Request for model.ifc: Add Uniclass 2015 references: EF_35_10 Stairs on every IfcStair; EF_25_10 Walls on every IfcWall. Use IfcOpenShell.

First a look at what the model holds.

```python
import ifcopenshell

model = ifcopenshell.open("model.ifc")
print(model.schema)
print("classifications:", [c.Name for c in model.by_type("IfcClassification")])
for ifc_class in ("IfcDoor", "IfcRoof", "IfcStair", "IfcWall", "IfcWindow"):
    print(ifc_class, len(model.by_type(ifc_class)))
```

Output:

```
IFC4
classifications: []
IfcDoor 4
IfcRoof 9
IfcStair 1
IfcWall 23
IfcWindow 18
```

```python
import ifcopenshell
import ifcopenshell.api.classification

model = ifcopenshell.open("model.ifc")

system = ifcopenshell.api.classification.add_classification(model, classification="Uniclass 2015")

codes = {
    "IfcStair": ("EF_35_10", "Stairs"),
    "IfcWall": ("EF_25_10", "Walls"),
}
for ifc_class, (code, name) in codes.items():
    products = model.by_type(ifc_class)
    ifcopenshell.api.classification.add_reference(
        model, products=products, classification=system, identification=code, name=name
    )
    print(code, len(products))

model.write("model-out.ifc")
```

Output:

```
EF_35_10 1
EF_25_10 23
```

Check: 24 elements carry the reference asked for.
